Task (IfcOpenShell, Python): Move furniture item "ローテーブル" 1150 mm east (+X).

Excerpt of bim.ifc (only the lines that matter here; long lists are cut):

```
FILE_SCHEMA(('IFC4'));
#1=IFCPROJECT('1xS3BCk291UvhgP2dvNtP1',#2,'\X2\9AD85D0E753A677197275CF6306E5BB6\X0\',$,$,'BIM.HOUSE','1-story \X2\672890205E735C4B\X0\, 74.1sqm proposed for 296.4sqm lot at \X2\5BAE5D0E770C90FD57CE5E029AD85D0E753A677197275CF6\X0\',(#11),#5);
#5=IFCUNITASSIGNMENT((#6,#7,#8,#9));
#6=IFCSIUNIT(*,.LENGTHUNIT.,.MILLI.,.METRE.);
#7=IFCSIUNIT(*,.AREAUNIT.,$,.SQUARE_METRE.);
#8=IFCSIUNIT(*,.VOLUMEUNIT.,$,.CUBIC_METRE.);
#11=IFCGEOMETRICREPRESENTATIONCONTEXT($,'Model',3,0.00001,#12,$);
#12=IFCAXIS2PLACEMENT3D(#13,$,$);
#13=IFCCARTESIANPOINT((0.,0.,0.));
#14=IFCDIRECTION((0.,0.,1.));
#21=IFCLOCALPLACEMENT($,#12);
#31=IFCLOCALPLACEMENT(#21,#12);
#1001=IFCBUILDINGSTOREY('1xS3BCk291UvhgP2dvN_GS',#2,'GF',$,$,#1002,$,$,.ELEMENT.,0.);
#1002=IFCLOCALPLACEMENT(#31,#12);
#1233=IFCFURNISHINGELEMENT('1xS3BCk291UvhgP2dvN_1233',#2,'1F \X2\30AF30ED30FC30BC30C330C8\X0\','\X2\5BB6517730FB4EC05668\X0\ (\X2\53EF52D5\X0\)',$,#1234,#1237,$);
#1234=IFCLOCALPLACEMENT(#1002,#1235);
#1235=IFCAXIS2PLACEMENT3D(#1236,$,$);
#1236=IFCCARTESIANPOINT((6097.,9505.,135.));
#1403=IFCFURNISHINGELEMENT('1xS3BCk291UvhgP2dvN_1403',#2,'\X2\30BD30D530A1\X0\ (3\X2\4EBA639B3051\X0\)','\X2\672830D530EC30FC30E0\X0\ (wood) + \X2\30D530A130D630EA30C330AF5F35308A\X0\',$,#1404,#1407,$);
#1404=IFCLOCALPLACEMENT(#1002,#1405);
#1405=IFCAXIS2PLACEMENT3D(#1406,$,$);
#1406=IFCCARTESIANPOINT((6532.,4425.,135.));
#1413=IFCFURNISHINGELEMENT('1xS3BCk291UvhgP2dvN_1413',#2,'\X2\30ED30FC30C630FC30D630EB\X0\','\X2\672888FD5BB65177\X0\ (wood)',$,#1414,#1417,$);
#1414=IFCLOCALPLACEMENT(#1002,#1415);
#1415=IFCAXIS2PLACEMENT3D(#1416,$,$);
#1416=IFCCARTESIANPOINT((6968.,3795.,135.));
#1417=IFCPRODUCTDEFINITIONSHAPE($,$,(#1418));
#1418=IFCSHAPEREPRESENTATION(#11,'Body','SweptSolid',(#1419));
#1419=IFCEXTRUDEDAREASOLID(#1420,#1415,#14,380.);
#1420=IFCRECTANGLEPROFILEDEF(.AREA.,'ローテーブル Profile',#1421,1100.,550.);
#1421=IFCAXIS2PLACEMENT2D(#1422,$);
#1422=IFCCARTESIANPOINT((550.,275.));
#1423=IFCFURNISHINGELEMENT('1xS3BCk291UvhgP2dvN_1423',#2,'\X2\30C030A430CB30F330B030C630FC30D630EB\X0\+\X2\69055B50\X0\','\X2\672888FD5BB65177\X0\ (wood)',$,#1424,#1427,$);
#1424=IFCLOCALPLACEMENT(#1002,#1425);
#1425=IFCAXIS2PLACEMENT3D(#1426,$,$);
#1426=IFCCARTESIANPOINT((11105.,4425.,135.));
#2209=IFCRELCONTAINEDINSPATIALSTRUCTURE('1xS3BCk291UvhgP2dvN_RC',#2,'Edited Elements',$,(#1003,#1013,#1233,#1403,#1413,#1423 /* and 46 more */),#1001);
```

```python
import ifcopenshell
import ifcopenshell.api.geometry
import ifcopenshell.util.placement
import ifcopenshell.util.unit

model = ifcopenshell.open("bim.ifc")
unit_scale = ifcopenshell.util.unit.calculate_unit_scale(model)

item = model.by_guid("1xS3BCk291UvhgP2dvN_1413")
matrix = ifcopenshell.util.placement.get_local_placement(item.ObjectPlacement)
matrix[0, 3] += 1.15 / unit_scale
ifcopenshell.api.geometry.edit_object_placement(model, product=item, matrix=matrix, is_si=False)

print(ifcopenshell.util.placement.get_local_placement(item.ObjectPlacement).round(3) + 0.0)

model.write("bim_edited.ifc")
```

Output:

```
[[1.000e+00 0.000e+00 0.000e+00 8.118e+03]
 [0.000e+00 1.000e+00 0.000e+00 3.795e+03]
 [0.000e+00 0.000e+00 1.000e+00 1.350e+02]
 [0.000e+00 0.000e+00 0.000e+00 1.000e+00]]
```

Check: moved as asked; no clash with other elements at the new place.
